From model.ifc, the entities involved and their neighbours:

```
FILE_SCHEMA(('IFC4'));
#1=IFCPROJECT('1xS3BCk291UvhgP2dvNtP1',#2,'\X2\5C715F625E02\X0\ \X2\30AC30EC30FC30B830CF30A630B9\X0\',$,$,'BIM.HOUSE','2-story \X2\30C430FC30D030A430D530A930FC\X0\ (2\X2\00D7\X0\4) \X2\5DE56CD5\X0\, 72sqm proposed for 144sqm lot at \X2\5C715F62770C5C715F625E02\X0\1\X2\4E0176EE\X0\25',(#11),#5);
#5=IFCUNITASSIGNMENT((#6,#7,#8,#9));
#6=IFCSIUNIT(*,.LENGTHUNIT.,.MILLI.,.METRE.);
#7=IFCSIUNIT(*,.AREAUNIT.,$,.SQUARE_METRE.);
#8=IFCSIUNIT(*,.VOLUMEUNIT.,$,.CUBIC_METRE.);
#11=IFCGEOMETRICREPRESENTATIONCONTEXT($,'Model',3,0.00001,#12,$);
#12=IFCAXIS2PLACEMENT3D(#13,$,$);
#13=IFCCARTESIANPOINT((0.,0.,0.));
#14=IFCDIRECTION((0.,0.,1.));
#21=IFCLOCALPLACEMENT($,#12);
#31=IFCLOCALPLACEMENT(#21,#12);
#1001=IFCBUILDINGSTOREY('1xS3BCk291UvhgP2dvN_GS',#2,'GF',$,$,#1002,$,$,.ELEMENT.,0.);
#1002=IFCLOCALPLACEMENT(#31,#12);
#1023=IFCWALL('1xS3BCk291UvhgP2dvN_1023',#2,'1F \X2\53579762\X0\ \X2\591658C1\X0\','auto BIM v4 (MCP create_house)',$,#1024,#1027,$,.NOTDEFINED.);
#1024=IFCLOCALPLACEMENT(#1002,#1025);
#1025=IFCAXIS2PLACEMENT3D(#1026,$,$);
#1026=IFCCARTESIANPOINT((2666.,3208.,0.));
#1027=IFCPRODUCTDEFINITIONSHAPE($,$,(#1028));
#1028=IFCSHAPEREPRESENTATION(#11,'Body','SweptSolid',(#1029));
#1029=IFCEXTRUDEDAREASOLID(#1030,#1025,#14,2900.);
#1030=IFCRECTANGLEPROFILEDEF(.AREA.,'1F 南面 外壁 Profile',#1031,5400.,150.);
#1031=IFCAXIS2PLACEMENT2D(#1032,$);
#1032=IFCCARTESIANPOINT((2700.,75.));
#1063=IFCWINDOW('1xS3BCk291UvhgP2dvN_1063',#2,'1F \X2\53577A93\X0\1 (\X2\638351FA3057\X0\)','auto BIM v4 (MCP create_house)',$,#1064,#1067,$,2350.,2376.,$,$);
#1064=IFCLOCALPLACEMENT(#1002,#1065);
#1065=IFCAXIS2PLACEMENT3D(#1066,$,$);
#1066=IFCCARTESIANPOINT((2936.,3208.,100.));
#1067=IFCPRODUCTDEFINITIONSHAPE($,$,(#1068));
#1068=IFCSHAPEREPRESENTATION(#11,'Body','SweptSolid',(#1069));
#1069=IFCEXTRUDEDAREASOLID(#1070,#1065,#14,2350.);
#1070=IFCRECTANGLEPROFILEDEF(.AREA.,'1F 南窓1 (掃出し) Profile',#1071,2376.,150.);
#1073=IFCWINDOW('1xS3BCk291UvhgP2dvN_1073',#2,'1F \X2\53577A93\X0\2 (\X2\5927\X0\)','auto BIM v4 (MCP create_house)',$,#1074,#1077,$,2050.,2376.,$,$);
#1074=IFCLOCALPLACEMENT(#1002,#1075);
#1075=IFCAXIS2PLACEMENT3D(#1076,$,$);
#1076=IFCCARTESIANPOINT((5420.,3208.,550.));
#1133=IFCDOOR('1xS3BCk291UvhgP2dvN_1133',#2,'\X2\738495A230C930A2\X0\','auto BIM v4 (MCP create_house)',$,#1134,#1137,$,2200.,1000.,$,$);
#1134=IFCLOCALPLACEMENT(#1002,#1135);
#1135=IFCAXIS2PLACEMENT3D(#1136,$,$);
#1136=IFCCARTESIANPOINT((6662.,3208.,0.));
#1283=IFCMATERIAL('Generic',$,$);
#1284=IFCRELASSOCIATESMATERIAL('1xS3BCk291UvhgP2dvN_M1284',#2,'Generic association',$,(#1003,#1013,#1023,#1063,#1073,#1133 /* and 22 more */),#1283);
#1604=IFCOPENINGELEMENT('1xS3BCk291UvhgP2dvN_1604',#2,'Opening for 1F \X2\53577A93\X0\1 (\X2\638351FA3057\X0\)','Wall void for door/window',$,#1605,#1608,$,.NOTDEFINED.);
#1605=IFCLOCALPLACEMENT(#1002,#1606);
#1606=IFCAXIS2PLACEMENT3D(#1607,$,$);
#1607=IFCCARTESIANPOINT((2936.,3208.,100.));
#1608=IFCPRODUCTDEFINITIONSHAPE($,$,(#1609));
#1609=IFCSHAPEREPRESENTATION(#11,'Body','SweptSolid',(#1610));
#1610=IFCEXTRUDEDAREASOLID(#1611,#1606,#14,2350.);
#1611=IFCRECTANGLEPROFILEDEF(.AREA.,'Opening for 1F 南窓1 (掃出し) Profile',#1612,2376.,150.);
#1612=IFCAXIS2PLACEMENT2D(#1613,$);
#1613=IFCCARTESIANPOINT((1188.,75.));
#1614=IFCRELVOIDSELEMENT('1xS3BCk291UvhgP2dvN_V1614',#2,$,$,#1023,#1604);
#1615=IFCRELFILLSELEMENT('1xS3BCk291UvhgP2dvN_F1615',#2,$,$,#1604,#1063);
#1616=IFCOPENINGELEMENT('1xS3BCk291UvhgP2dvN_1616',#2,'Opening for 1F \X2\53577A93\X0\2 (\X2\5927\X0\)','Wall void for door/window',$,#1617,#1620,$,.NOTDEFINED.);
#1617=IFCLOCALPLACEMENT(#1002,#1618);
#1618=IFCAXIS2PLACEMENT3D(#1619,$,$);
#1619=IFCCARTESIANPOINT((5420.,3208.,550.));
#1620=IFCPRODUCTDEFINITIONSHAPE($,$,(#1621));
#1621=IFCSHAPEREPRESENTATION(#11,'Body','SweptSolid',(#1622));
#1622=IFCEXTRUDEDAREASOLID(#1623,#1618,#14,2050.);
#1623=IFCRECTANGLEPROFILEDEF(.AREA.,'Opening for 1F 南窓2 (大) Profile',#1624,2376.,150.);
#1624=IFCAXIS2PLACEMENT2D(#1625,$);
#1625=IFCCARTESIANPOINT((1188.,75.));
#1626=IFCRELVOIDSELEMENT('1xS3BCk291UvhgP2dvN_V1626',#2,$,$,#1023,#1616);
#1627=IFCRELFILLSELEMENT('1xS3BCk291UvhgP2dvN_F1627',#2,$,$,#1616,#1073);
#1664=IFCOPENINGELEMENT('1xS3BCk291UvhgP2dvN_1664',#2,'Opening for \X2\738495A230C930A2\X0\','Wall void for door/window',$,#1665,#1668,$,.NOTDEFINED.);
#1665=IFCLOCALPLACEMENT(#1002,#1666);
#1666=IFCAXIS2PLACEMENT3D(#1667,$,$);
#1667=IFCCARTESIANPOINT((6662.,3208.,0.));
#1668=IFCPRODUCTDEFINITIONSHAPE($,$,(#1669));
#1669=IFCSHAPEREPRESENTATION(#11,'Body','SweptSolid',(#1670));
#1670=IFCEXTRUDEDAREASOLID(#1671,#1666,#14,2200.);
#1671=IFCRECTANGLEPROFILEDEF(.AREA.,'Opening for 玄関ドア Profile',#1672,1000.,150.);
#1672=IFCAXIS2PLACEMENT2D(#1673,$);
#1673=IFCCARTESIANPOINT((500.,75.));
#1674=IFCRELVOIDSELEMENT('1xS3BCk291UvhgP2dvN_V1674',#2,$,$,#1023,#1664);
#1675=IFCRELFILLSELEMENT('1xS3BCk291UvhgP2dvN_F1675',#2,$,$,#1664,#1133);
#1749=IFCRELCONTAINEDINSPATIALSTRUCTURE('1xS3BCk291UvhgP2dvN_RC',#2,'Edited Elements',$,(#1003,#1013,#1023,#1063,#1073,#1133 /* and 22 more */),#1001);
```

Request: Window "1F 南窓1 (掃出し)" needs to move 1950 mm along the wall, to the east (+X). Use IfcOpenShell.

```python
import ifcopenshell
import ifcopenshell.api.geometry
import ifcopenshell.util.placement
import ifcopenshell.util.unit

model = ifcopenshell.open("model.ifc")
unit_scale = ifcopenshell.util.unit.calculate_unit_scale(model)

window = model.by_id(1063)
opening = window.FillsVoids[0].RelatingOpeningElement
wall = opening.VoidsElements[0].RelatingBuildingElement

wall_matrix = ifcopenshell.util.placement.get_local_placement(wall.ObjectPlacement)
shift = wall_matrix[:3, 0] * 1.95 / unit_scale
before = ifcopenshell.util.placement.get_local_placement(window.ObjectPlacement)[:3, 3].copy()

# The window is not placed relative to its opening, so move both.
for product in (opening, window):
    matrix = ifcopenshell.util.placement.get_local_placement(product.ObjectPlacement)
    matrix[:3, 3] += shift
    ifcopenshell.api.geometry.edit_object_placement(model, product=product, matrix=matrix, is_si=False)

after = ifcopenshell.util.placement.get_local_placement(window.ObjectPlacement)[:3, 3]
print("window moved by", (after - before).round(3) + 0.0)

model.write("model_rev.ifc")
```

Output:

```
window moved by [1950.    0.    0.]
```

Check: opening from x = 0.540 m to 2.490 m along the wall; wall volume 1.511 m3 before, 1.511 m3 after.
